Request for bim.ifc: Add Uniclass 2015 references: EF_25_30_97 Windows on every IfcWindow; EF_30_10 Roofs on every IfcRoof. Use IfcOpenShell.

First a look at what the model holds.

```python
import ifcopenshell

model = ifcopenshell.open("bim.ifc")
print(model.schema)
print("classifications:", [c.Name for c in model.by_type("IfcClassification")])
for ifc_class in ("IfcDoor", "IfcRoof", "IfcStair", "IfcWall", "IfcWindow"):
    print(ifc_class, len(model.by_type(ifc_class)))
```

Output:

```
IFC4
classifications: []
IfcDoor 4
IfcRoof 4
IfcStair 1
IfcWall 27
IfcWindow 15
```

```python
import ifcopenshell
import ifcopenshell.api.classification

model = ifcopenshell.open("bim.ifc")

system = ifcopenshell.api.classification.add_classification(model, classification="Uniclass 2015")

codes = {
    "IfcWindow": ("EF_25_30_97", "Windows"),
    "IfcRoof": ("EF_30_10", "Roofs"),
}
for ifc_class, (code, name) in codes.items():
    products = model.by_type(ifc_class)
    ifcopenshell.api.classification.add_reference(
        model, products=products, classification=system, identification=code, name=name
    )
    print(code, len(products))

model.write("bim_v2.ifc")
```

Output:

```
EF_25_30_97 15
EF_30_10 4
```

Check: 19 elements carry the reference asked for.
